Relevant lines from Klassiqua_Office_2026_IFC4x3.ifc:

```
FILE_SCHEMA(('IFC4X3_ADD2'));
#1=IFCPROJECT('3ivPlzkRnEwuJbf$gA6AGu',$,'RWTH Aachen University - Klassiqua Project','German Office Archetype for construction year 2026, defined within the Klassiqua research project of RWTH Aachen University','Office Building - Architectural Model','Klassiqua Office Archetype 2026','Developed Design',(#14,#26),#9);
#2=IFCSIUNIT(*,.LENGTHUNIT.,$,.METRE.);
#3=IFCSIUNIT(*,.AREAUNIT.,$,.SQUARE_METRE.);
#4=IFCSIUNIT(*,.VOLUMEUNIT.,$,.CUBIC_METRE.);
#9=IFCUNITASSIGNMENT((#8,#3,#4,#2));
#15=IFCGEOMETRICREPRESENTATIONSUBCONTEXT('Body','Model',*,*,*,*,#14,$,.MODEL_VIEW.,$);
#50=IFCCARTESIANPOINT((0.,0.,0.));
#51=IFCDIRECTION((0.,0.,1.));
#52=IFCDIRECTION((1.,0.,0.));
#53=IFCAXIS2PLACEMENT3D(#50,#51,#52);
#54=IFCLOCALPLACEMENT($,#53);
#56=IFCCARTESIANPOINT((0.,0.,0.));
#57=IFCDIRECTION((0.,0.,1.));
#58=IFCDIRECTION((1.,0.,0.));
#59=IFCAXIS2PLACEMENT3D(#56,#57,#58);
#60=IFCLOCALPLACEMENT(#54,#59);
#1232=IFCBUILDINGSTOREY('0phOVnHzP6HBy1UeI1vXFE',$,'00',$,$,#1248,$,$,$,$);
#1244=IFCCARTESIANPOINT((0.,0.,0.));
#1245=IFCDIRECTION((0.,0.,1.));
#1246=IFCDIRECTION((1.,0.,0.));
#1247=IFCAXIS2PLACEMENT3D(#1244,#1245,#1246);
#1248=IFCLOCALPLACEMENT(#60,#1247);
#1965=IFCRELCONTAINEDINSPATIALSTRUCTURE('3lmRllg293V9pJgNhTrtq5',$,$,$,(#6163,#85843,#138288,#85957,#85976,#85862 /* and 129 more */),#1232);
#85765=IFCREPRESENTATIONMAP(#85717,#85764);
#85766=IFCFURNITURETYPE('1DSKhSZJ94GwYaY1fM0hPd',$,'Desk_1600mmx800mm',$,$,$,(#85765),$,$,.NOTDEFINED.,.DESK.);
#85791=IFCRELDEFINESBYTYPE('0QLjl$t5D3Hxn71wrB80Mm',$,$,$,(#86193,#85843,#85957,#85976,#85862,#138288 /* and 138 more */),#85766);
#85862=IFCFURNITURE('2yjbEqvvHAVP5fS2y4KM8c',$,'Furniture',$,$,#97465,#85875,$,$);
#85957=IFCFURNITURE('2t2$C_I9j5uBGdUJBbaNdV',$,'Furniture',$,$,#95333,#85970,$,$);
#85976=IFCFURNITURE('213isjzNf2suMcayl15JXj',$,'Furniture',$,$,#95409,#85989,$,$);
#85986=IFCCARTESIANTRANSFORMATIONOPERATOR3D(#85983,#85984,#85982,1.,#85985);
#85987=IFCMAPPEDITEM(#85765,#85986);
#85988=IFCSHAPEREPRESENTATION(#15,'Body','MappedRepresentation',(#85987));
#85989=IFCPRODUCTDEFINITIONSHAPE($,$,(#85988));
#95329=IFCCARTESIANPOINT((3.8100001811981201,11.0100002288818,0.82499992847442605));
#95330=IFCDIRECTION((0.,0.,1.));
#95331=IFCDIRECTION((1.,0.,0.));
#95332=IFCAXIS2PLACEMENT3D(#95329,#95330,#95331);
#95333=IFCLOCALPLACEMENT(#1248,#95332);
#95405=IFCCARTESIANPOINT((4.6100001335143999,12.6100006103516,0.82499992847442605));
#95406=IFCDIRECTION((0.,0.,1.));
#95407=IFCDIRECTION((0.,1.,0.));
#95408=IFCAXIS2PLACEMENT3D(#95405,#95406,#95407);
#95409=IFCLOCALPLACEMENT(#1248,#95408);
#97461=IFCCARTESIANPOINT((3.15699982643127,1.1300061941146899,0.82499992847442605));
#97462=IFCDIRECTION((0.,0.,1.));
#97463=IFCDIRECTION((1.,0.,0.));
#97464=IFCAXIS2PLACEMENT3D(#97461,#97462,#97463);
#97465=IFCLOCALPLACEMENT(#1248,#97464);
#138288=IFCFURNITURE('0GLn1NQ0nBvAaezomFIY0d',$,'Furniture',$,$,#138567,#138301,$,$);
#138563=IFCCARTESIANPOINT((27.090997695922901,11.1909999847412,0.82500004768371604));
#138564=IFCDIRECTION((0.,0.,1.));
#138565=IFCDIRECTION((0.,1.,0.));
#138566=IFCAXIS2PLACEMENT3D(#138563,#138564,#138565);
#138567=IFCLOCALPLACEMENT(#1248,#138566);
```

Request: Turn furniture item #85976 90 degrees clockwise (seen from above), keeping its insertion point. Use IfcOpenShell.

```python
import ifcopenshell
import ifcopenshell.api.geometry
import ifcopenshell.util.placement

model = ifcopenshell.open("Klassiqua_Office_2026_IFC4x3.ifc")

item = model.by_id(85976)
matrix = ifcopenshell.util.placement.get_local_placement(item.ObjectPlacement)
matrix = matrix @ ifcopenshell.util.placement.rotation(-90, "Z")
ifcopenshell.api.geometry.edit_object_placement(model, product=item, matrix=matrix, is_si=False)

print(ifcopenshell.util.placement.get_local_placement(item.ObjectPlacement).round(3) + 0.0)

model.write("Klassiqua_Office_2026_IFC4x3_updated.ifc")
```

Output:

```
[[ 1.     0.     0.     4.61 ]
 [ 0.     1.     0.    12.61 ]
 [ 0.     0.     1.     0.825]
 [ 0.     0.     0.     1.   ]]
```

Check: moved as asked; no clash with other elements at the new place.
